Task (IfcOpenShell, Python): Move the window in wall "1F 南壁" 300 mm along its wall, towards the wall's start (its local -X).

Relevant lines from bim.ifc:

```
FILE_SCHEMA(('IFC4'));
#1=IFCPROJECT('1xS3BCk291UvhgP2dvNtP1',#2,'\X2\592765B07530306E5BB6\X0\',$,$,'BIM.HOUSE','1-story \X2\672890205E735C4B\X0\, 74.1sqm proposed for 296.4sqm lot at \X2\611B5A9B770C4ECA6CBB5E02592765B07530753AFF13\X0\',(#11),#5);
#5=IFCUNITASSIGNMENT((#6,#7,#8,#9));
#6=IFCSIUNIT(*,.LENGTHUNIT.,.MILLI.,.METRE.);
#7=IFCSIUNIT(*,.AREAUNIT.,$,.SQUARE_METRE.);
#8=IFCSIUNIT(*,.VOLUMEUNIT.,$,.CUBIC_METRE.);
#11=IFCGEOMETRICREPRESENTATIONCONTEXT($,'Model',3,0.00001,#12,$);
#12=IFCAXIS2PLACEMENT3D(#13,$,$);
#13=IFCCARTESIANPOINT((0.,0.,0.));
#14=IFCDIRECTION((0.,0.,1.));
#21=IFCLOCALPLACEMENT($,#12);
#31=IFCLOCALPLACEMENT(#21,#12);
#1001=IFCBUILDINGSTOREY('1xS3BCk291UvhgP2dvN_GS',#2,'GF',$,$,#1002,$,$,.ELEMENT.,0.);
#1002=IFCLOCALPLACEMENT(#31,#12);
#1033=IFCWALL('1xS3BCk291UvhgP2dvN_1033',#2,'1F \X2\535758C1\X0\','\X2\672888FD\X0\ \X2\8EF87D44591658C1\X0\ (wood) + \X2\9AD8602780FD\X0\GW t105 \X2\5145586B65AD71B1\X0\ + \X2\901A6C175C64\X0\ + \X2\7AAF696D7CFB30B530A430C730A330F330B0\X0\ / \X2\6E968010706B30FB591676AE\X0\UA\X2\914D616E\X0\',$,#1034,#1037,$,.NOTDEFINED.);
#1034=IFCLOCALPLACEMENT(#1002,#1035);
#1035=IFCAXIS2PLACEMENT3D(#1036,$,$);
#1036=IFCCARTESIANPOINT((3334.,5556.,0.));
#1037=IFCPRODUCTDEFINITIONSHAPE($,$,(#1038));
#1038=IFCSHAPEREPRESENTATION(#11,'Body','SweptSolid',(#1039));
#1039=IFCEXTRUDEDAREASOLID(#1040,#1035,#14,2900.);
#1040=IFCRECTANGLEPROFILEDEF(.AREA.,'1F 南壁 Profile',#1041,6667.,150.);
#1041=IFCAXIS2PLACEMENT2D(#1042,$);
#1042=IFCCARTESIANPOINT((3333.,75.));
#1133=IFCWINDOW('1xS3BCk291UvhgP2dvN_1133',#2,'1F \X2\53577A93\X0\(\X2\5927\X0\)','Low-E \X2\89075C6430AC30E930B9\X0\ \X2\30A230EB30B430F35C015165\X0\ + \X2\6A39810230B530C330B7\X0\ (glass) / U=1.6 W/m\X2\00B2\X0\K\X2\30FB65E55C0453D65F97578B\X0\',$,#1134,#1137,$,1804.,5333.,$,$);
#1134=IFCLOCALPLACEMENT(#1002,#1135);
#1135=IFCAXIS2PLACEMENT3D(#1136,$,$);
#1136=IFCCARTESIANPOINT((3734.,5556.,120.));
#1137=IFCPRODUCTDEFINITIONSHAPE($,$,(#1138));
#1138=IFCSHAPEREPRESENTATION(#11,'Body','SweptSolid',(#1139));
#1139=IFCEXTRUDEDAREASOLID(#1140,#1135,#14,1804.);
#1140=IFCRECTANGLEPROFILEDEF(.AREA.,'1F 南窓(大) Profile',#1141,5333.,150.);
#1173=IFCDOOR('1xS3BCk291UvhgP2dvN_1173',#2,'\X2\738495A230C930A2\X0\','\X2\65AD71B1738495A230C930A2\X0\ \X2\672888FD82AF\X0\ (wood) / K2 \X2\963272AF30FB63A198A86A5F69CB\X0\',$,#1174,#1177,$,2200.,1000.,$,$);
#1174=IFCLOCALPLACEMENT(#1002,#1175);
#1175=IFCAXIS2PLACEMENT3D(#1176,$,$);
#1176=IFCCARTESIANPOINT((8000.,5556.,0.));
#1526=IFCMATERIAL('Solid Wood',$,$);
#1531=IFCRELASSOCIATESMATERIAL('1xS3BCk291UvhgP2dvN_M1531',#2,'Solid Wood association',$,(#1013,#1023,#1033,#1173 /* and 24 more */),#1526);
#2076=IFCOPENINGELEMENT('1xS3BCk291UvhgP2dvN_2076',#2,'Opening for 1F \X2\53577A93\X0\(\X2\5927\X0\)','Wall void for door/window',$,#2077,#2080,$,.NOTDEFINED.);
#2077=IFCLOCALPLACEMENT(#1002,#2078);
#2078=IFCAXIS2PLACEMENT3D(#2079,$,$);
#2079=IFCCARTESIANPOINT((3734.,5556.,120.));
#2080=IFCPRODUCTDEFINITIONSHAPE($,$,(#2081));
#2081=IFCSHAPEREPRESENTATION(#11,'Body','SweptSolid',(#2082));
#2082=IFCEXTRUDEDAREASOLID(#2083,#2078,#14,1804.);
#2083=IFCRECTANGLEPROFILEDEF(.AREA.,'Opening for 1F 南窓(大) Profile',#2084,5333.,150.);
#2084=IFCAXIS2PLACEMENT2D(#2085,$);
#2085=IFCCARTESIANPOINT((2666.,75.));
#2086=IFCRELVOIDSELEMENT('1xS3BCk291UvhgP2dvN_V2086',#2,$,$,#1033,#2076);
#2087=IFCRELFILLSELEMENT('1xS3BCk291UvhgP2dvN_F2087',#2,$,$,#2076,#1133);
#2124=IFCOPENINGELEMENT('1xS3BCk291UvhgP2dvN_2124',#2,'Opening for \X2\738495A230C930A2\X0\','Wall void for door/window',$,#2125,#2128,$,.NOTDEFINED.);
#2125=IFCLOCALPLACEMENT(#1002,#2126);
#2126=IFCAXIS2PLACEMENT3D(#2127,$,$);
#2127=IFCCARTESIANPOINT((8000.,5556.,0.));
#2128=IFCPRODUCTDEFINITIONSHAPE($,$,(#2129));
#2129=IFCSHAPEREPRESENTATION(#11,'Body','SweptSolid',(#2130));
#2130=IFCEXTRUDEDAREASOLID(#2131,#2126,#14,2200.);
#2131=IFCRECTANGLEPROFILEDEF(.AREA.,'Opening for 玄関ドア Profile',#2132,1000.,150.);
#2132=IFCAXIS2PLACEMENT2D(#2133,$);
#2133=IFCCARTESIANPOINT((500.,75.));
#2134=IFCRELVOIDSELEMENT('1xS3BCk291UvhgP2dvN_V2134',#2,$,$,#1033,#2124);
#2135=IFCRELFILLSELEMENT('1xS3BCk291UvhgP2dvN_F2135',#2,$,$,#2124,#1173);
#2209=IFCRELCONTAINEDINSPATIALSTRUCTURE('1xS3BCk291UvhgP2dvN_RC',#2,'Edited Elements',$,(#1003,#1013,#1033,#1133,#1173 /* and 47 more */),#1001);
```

```python
import ifcopenshell
import ifcopenshell.api.geometry
import ifcopenshell.util.placement
import ifcopenshell.util.unit

model = ifcopenshell.open("bim.ifc")
unit_scale = ifcopenshell.util.unit.calculate_unit_scale(model)

window = model.by_guid("1xS3BCk291UvhgP2dvN_1133")
opening = window.FillsVoids[0].RelatingOpeningElement
wall = opening.VoidsElements[0].RelatingBuildingElement

wall_matrix = ifcopenshell.util.placement.get_local_placement(wall.ObjectPlacement)
shift = wall_matrix[:3, 0] * -0.3 / unit_scale
before = ifcopenshell.util.placement.get_local_placement(window.ObjectPlacement)[:3, 3].copy()

# The window is not placed relative to its opening, so move both.
for product in (opening, window):
    matrix = ifcopenshell.util.placement.get_local_placement(product.ObjectPlacement)
    matrix[:3, 3] += shift
    ifcopenshell.api.geometry.edit_object_placement(model, product=product, matrix=matrix, is_si=False)

after = ifcopenshell.util.placement.get_local_placement(window.ObjectPlacement)[:3, 3]
print("window moved by", (after - before).round(3) + 0.0)

model.write("bim_v2.ifc")
```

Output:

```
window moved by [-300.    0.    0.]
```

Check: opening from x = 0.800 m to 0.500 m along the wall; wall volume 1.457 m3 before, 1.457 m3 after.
